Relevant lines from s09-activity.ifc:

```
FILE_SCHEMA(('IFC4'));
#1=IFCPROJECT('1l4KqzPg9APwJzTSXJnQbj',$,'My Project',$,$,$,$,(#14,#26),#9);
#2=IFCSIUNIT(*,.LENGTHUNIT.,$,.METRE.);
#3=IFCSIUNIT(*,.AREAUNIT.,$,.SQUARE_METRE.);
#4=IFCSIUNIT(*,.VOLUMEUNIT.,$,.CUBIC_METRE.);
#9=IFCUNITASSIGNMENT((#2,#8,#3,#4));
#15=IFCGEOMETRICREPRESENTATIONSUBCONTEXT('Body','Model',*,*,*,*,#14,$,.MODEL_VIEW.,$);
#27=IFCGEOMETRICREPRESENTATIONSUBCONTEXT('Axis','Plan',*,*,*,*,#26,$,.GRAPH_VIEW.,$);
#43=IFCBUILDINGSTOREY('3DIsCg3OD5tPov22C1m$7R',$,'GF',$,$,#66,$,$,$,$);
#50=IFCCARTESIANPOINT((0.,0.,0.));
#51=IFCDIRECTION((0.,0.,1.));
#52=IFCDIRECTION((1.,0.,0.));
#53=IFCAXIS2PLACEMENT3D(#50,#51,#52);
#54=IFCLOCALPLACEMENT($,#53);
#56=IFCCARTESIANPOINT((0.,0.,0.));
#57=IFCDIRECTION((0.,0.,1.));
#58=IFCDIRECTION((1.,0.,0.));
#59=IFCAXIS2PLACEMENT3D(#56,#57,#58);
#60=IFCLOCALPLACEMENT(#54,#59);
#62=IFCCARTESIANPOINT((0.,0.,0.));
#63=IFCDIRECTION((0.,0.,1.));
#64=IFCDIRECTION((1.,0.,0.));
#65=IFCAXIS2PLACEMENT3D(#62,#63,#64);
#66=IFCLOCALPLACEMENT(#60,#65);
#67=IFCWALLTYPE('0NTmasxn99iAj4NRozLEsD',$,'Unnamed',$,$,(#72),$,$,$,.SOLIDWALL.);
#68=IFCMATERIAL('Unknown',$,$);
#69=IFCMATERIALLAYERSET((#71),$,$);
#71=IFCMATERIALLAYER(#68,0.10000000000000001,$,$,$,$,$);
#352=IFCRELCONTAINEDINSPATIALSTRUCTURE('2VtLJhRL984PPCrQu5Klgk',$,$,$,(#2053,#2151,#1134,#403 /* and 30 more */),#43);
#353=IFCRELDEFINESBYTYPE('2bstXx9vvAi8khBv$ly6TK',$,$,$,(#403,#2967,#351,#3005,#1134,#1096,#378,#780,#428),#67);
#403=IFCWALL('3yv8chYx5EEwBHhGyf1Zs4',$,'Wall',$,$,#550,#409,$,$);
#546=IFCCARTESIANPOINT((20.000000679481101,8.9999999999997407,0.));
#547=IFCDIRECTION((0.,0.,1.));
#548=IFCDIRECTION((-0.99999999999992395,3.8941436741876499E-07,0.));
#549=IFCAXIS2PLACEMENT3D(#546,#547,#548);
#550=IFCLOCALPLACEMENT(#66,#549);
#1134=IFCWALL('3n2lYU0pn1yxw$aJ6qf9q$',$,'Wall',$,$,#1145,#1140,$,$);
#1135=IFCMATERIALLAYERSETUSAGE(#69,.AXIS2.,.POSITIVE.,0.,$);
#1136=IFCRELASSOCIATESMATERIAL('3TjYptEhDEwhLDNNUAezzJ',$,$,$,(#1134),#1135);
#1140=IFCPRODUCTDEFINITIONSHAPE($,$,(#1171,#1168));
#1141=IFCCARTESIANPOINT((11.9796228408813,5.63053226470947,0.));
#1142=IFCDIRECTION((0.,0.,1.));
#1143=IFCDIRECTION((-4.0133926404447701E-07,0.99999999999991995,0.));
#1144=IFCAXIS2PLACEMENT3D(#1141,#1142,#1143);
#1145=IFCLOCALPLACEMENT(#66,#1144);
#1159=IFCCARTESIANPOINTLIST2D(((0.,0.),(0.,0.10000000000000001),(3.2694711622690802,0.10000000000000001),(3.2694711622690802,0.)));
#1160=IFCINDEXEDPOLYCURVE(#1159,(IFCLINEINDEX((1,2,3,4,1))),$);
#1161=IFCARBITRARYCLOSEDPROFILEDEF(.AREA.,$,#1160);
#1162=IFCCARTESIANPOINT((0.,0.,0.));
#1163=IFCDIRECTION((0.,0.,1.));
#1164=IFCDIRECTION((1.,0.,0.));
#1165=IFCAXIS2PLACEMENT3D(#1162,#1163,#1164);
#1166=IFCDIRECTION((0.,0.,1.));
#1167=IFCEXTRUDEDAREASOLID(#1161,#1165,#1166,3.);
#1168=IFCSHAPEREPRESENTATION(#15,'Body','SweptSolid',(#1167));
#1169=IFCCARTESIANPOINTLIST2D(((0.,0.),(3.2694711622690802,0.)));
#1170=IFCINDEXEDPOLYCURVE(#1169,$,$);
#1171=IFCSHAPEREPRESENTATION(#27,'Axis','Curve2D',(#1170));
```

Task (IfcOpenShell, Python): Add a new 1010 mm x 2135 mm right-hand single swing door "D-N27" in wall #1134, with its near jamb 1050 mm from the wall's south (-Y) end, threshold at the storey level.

```python
import numpy as np
import ifcopenshell
import ifcopenshell.api.feature
import ifcopenshell.api.geometry
import ifcopenshell.api.root
import ifcopenshell.api.spatial
import ifcopenshell.geom
import ifcopenshell.util.element
import ifcopenshell.util.placement
import ifcopenshell.util.representation
import ifcopenshell.util.shape
import ifcopenshell.util.unit

model = ifcopenshell.open("s09-activity.ifc")
unit_scale = ifcopenshell.util.unit.calculate_unit_scale(model)
settings = ifcopenshell.geom.settings()


def volume(element):
    """Net volume in cubic metres, openings subtracted."""
    shape = ifcopenshell.geom.create_shape(settings, element)
    return ifcopenshell.util.shape.get_volume(shape.geometry)


wall = model.by_guid("3n2lYU0pn1yxw$aJ6qf9q$")
storey = ifcopenshell.util.element.get_container(wall, ifc_class="IfcBuildingStorey")
context = ifcopenshell.util.representation.get_context(model, "Model", "Body", "MODEL_VIEW")
before = volume(wall)

width, height, from_end, sill = 1.01, 2.135, 1.05, 0.0  # metres

# The wall runs along its own X axis, and the end named is its -X end.
wall_shape = ifcopenshell.geom.create_shape(settings, wall)
x, y, z = ifcopenshell.util.shape.get_vertices(wall_shape.geometry).T
start = x.min() + from_end
face, thickness = float(y.min()), float(y.max() - y.min())
wall_matrix = ifcopenshell.util.placement.get_local_placement(wall.ObjectPlacement)
level = ifcopenshell.util.placement.get_local_placement(storey.ObjectPlacement)[2, 3]


def in_wall(x, y):
    """Placement at x, y metres in the wall's axes, at sill height."""
    matrix = wall_matrix.copy()
    matrix[:, 3] = wall_matrix @ np.array([x / unit_scale, y / unit_scale, 0.0, 1.0])
    matrix[2, 3] = level + sill / unit_scale
    return matrix


# Opening: a box that overshoots both wall faces by 50 mm.
opening = ifcopenshell.api.root.create_entity(model, ifc_class="IfcOpeningElement", predefined_type="OPENING")
box = ifcopenshell.api.geometry.add_wall_representation(
    model, context=context, length=width, height=height, thickness=thickness + 0.1
)
ifcopenshell.api.geometry.assign_representation(model, product=opening, representation=box)
ifcopenshell.api.geometry.edit_object_placement(model, product=opening, matrix=in_wall(start, face - 0.05), is_si=False)
ifcopenshell.api.feature.add_feature(model, feature=opening, element=wall)

door = ifcopenshell.api.root.create_entity(model, ifc_class="IfcDoor", name="D-N27", predefined_type="DOOR")
door.OverallWidth, door.OverallHeight = width / unit_scale, height / unit_scale
door.OperationType = "SINGLE_SWING_RIGHT"
body = ifcopenshell.api.geometry.add_door_representation(
    model,
    context=context,
    overall_width=door.OverallWidth,
    overall_height=door.OverallHeight,
    operation_type="SINGLE_SWING_RIGHT",
    lining_properties={"LiningDepth": thickness / unit_scale, "ThresholdDepth": thickness / unit_scale},
)
ifcopenshell.api.geometry.assign_representation(model, product=door, representation=body)
ifcopenshell.api.spatial.assign_container(model, products=[door], relating_structure=storey)
ifcopenshell.api.feature.add_filling(model, opening=opening, element=door)

# The lining spans the wall, so the door starts at the wall face.
ifcopenshell.api.geometry.edit_object_placement(model, product=door, matrix=in_wall(start, face), is_si=False)

after = volume(wall)

print(f"wall volume {before:.3f} -> {after:.3f} m3")

model.write("s09-activity-out.ifc")
```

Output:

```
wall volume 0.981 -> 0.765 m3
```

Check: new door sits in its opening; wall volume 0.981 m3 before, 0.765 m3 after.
